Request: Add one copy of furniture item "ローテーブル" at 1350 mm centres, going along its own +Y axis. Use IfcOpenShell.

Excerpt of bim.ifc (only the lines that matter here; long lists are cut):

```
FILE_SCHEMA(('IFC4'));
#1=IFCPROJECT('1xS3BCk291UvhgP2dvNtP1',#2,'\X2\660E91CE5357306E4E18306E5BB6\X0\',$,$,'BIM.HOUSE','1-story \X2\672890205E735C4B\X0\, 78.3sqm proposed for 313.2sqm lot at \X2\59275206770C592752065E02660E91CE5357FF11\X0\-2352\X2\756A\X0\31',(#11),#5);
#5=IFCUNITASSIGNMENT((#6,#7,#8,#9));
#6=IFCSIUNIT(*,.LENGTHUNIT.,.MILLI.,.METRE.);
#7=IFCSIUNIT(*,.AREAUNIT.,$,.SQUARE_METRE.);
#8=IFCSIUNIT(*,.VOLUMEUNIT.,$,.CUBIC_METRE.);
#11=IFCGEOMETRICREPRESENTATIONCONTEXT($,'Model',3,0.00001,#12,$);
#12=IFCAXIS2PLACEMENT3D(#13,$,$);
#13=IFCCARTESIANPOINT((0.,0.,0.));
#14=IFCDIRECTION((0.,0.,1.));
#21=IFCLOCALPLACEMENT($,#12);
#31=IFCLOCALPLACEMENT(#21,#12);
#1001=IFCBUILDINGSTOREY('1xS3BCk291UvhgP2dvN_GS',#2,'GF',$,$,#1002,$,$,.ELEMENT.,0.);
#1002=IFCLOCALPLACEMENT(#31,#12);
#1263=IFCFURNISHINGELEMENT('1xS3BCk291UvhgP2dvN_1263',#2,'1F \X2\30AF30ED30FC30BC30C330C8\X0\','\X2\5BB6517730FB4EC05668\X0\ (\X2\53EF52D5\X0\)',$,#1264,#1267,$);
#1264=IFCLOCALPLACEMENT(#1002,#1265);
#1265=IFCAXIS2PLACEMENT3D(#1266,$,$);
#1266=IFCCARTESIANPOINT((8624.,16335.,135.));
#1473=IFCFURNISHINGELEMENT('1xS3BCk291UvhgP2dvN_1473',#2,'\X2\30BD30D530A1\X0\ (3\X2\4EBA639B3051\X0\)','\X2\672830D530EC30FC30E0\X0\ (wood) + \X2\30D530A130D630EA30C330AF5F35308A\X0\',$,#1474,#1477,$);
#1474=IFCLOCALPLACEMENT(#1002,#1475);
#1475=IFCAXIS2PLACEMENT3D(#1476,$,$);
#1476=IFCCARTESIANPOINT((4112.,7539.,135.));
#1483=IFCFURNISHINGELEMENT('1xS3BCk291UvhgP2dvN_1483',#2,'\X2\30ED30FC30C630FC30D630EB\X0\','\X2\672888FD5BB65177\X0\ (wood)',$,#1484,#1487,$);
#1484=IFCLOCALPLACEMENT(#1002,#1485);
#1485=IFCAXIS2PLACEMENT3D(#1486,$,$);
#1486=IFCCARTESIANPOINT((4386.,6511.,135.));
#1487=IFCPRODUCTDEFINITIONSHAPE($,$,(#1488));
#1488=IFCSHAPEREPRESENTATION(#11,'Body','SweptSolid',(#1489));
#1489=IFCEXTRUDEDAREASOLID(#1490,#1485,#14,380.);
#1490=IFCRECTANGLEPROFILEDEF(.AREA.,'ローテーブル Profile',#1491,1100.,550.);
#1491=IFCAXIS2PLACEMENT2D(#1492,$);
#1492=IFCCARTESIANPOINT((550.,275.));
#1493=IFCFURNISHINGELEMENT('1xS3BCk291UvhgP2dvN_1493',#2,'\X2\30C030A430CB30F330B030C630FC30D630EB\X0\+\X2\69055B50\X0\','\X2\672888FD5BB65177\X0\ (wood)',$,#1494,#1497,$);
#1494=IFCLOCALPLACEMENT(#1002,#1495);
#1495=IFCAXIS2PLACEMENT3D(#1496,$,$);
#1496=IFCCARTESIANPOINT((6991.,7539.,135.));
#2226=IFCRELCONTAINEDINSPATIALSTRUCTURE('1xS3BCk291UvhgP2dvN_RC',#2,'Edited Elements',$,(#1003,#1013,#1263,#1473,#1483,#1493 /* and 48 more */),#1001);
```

```python
import ifcopenshell
import ifcopenshell.api.geometry
import ifcopenshell.api.root
import ifcopenshell.util.element
import ifcopenshell.util.placement
import ifcopenshell.util.unit

model = ifcopenshell.open("bim.ifc")
unit_scale = ifcopenshell.util.unit.calculate_unit_scale(model)


def reuse_history(source, copy):
    """copy_class also copies each property set's owner history, people and application; keep the originals."""
    for rel in copy.IsDefinedBy:
        if rel.is_a("IfcRelDefinesByProperties") and (history := rel.RelatingPropertyDefinition.OwnerHistory):
            rel.RelatingPropertyDefinition.OwnerHistory = source.OwnerHistory
            ifcopenshell.util.element.remove_deep2(model, history)


source = model.by_guid("1xS3BCk291UvhgP2dvN_1483")
base = ifcopenshell.util.placement.get_local_placement(source.ObjectPlacement)
step = base[:3, 1] * 1.35 / unit_scale

for i in range(1, 2):
    copy = ifcopenshell.api.root.copy_class(model, product=source)
    copy.Representation = ifcopenshell.util.element.copy_deep(
        model, source.Representation, exclude=["IfcGeometricRepresentationContext", "IfcRepresentationMap"]
    )
    reuse_history(source, copy)
    matrix = base.copy()
    matrix[:3, 3] += i * step
    print("added at", matrix[:3, 3].round(3) + 0.0)
    ifcopenshell.api.geometry.edit_object_placement(model, product=copy, matrix=matrix, is_si=False)

model.write("bim-out.ifc")
```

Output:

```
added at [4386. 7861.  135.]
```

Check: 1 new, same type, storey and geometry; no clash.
